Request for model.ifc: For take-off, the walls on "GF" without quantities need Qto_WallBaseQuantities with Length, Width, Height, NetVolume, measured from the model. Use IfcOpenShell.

First a look at what the model holds.

```python
import ifcopenshell
import ifcopenshell.util.element
import ifcopenshell.util.unit

model = ifcopenshell.open("model.ifc")
print(model.schema)
for unit_type in ("LENGTHUNIT", "AREAUNIT", "VOLUMEUNIT"):
    print(unit_type, ifcopenshell.util.unit.calculate_unit_scale(model, unit_type))
storey = next(s for s in model.by_type("IfcBuildingStorey") if s.Name == "GF")
walls = [e for e in ifcopenshell.util.element.get_decomposition(storey) if e.is_a("IfcWall")]
for e in sorted(walls, key=lambda e: e.id()):
    print(e.id(), e.is_a(), e.Name, list(ifcopenshell.util.element.get_psets(e, qtos_only=True)), sep=" | ")
```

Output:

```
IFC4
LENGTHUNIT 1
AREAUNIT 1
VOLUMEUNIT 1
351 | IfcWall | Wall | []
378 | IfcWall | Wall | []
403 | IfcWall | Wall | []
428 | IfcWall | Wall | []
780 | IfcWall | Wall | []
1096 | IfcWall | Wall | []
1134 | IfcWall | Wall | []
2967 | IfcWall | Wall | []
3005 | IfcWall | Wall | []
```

```python
import ifcopenshell
import ifcopenshell.api.pset
import ifcopenshell.geom
import ifcopenshell.util.element
import ifcopenshell.util.shape
import ifcopenshell.util.unit

model = ifcopenshell.open("model.ifc")
unit_scale = ifcopenshell.util.unit.calculate_unit_scale(model)
volume_scale = ifcopenshell.util.unit.calculate_unit_scale(model, "VOLUMEUNIT")
settings = ifcopenshell.geom.settings()

storey = next(s for s in model.by_type("IfcBuildingStorey") if s.Name == "GF")
walls = [e for e in ifcopenshell.util.element.get_decomposition(storey) if e.is_a("IfcWall")]

for e in sorted(walls, key=lambda e: e.id()):
    if ifcopenshell.util.element.get_psets(e, qtos_only=True, should_inherit=False):
        continue
    # Geometry comes back in metres, in the element's own axes.
    shape = ifcopenshell.geom.create_shape(settings, e)
    values = {
        "Length": ifcopenshell.util.shape.get_x(shape.geometry) / unit_scale,
        "Width": ifcopenshell.util.shape.get_y(shape.geometry) / unit_scale,
        "Height": ifcopenshell.util.shape.get_z(shape.geometry) / unit_scale,
        "NetVolume": ifcopenshell.util.shape.get_volume(shape.geometry) / volume_scale,
    }
    qto = ifcopenshell.api.pset.add_qto(model, product=e, name="Qto_WallBaseQuantities")
    ifcopenshell.api.pset.edit_qto(model, qto=qto, properties=values)
    print(e.id(), {k: round(v, 3) for k, v in values.items()})

model.write("model-out.ifc")
```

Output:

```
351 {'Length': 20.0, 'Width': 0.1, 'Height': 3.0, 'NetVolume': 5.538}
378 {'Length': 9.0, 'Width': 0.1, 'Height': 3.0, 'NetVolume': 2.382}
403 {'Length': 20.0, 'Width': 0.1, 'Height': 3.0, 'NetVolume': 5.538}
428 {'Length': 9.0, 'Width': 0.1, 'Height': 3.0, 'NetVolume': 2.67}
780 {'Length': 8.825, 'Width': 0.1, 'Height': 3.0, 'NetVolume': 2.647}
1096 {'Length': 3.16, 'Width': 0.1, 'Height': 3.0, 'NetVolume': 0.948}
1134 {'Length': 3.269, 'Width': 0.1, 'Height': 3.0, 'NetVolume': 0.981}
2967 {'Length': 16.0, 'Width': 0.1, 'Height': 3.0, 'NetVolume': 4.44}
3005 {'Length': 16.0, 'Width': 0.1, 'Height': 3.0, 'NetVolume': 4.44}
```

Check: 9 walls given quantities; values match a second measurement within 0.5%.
